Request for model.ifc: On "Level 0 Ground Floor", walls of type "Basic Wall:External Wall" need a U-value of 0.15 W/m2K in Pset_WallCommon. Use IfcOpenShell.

First a look at what the model holds.

```python
import ifcopenshell
import ifcopenshell.util.element

model = ifcopenshell.open("model.ifc")
print(model.schema)
storey = next(s for s in model.by_type("IfcBuildingStorey") if s.Name == "Level 0 Ground Floor")
walls = [e for e in ifcopenshell.util.element.get_decomposition(storey) if e.is_a("IfcWall")]
seen = {}
for e in walls:
    element_type = ifcopenshell.util.element.get_type(e)
    key = (element_type.Name if element_type != e and element_type else None, ifcopenshell.util.element.get_pset(e, "Pset_WallCommon", "ThermalTransmittance"))
    seen[key] = seen.get(key, 0) + 1
for (name, value), count in sorted(seen.items(), key=str):
    print(count, "x", name, "|", value)
```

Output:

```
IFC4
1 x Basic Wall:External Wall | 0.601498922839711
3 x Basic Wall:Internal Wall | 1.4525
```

```python
import ifcopenshell
import ifcopenshell.api.pset
import ifcopenshell.util.element

model = ifcopenshell.open("model.ifc")

storey = next(s for s in model.by_type("IfcBuildingStorey") if s.Name == "Level 0 Ground Floor")
walls = [e for e in ifcopenshell.util.element.get_decomposition(storey) if e.is_a("IfcWall")]

count = 0
for e in walls:
    element_type = ifcopenshell.util.element.get_type(e)
    if element_type in (None, e) or element_type.Name != "Basic Wall:External Wall":
        continue
    # add_pset returns the element's existing set when there is one.
    pset = ifcopenshell.api.pset.add_pset(model, product=e, name="Pset_WallCommon")
    ifcopenshell.api.pset.edit_pset(model, pset=pset, properties={"ThermalTransmittance": 0.15})
    count += 1

print(count, "walls updated")

model.write("model_edited.ifc")
```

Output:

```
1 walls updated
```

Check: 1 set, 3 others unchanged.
